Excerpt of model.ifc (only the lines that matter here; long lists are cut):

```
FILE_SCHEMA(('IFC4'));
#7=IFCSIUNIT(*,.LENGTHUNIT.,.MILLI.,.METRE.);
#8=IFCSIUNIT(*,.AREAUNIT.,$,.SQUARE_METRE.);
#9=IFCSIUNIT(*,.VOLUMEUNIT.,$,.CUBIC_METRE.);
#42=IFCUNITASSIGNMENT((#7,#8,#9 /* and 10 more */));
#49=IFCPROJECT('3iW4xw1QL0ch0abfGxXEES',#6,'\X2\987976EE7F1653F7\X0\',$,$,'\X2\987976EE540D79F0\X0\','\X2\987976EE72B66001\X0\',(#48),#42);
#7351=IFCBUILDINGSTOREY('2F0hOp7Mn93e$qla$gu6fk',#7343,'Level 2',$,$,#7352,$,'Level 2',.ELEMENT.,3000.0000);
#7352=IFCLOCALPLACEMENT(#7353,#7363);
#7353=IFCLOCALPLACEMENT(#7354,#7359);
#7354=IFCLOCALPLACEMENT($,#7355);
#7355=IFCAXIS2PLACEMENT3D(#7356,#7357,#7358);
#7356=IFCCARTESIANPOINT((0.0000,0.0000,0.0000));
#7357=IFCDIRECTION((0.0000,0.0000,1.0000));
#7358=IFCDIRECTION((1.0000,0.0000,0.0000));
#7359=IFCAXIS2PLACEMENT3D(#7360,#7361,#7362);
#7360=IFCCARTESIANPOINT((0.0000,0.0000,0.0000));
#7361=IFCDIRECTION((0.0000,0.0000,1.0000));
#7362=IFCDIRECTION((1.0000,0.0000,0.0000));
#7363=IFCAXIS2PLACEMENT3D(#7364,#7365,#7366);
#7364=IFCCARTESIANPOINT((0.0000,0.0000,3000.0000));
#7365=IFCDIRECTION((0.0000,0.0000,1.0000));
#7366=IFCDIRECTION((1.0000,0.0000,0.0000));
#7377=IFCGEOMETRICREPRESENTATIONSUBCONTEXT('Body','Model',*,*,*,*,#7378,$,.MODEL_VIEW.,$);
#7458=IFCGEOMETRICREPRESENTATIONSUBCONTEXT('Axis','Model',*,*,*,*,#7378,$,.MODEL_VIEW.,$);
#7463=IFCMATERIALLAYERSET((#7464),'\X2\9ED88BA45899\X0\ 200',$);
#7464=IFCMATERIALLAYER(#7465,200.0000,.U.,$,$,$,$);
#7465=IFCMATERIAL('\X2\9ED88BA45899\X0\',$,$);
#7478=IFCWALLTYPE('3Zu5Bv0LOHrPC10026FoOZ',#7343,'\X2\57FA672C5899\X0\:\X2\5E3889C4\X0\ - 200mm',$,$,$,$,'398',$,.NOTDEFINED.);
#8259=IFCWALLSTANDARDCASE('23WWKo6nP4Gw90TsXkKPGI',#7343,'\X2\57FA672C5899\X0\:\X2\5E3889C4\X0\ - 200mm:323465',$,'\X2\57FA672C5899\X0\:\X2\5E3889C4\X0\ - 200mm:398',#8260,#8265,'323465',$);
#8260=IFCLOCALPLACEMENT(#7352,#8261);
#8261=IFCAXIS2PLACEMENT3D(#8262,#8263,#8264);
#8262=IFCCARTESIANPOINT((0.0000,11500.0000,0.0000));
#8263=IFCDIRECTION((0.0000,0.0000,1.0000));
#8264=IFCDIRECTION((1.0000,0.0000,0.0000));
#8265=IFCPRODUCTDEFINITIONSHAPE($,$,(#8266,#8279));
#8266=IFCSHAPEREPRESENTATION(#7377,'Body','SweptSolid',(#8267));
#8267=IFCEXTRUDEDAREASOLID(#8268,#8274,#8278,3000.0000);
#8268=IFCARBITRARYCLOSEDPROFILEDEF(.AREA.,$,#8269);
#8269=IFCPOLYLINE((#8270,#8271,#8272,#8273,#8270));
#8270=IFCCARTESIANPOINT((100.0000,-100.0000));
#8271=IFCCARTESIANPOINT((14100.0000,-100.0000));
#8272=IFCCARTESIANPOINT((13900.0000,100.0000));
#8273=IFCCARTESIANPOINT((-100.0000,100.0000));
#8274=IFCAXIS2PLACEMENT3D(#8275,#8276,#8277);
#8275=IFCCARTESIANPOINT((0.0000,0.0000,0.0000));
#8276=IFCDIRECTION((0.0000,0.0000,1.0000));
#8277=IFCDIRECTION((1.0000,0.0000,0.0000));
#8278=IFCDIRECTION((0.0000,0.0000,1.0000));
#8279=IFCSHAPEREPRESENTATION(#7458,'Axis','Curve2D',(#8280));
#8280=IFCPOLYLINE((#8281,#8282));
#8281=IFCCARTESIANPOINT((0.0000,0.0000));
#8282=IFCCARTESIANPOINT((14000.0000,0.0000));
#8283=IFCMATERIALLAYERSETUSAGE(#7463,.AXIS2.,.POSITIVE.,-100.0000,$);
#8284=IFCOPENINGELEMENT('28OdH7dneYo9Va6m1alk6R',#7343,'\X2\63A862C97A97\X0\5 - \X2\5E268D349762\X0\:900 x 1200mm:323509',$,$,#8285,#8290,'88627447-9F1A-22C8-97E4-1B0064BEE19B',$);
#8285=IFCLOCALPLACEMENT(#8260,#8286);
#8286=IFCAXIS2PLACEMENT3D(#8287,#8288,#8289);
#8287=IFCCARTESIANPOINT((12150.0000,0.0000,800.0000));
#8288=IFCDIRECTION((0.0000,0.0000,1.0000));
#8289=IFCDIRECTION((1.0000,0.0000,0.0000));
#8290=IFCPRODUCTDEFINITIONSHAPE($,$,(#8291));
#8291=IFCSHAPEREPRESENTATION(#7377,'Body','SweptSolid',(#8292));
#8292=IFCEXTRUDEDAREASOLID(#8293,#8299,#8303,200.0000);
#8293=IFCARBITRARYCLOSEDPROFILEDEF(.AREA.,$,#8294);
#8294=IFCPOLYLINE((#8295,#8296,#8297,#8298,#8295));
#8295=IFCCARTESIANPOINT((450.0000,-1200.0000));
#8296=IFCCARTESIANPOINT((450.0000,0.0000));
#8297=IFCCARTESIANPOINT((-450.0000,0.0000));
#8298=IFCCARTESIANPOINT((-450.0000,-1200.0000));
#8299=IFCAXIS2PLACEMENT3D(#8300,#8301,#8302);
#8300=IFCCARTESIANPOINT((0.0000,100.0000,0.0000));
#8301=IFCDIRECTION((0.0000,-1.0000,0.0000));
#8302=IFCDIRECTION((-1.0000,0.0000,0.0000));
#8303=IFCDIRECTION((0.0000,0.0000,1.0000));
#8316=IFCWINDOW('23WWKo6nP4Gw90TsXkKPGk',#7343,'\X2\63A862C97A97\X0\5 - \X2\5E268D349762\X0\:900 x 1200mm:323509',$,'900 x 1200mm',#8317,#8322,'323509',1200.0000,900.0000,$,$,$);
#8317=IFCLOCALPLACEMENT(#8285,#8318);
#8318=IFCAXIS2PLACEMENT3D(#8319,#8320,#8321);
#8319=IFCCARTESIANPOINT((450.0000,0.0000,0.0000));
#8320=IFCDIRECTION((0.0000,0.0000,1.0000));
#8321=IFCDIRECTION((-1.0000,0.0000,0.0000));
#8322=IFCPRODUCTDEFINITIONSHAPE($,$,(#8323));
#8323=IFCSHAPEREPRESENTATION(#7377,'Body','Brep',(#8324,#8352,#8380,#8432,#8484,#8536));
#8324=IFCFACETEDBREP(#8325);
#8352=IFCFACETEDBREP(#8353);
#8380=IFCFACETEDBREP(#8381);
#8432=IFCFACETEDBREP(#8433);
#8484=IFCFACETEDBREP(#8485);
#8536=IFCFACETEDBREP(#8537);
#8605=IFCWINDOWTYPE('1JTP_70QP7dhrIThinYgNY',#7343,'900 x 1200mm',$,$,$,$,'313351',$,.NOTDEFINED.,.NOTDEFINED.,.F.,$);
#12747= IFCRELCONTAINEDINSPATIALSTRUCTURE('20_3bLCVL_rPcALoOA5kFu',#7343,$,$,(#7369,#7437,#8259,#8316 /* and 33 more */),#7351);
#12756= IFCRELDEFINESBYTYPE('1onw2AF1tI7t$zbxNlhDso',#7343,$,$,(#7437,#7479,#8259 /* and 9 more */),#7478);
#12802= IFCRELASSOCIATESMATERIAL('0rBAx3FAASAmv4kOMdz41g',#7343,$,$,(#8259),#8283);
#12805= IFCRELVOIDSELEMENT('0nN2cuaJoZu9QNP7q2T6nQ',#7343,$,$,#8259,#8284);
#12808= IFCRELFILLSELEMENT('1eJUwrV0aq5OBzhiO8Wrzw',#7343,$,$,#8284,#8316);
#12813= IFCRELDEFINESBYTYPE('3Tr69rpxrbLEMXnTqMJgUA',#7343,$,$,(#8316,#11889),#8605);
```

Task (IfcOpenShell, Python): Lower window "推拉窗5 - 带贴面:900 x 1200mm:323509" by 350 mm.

```python
import numpy as np
import ifcopenshell
import ifcopenshell.api.geometry
import ifcopenshell.util.placement
import ifcopenshell.util.unit

model = ifcopenshell.open("model.ifc")
unit_scale = ifcopenshell.util.unit.calculate_unit_scale(model)

window = model.by_id(8316)
opening = window.FillsVoids[0].RelatingOpeningElement
dz = -0.35 / unit_scale

shift = np.array([0.0, 0.0, dz])
# The window is placed relative to its opening, so it follows when the opening moves.
matrix = ifcopenshell.util.placement.get_local_placement(opening.ObjectPlacement)
matrix[:3, 3] += shift
ifcopenshell.api.geometry.edit_object_placement(
    model, product=opening, matrix=matrix, is_si=False, should_transform_children=True
)

print(f"moved by {dz * unit_scale:+.3f} m")

model.write("model_rev.ifc")
```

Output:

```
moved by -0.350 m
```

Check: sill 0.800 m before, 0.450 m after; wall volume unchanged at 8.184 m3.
